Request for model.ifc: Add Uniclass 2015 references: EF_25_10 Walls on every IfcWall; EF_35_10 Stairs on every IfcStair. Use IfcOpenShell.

First a look at what the model holds.

```python
import ifcopenshell

model = ifcopenshell.open("model.ifc")
print(model.schema)
print("classifications:", [c.Name for c in model.by_type("IfcClassification")])
for ifc_class in ("IfcDoor", "IfcRoof", "IfcStair", "IfcWall", "IfcWindow"):
    print(ifc_class, len(model.by_type(ifc_class)))
```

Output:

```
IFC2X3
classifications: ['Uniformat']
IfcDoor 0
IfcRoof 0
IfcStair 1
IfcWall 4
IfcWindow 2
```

```python
import ifcopenshell
import ifcopenshell.api.classification

model = ifcopenshell.open("model.ifc")

# IFC2X3 requires Source and Edition and has no link from the project to the system.
system = model.create_entity("IfcClassification", Source="NBS", Edition="2015", Name="Uniclass 2015")

codes = {
    "IfcWall": ("EF_25_10", "Walls"),
    "IfcStair": ("EF_35_10", "Stairs"),
}
for ifc_class, (code, name) in codes.items():
    products = model.by_type(ifc_class)
    ifcopenshell.api.classification.add_reference(
        model, products=products, classification=system, identification=code, name=name
    )
    print(code, len(products))

model.write("model_updated.ifc")
```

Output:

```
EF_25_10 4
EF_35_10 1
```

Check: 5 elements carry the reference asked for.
